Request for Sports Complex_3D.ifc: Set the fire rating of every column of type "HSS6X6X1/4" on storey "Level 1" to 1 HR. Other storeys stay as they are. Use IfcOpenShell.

First a look at what the model holds.

```python
import ifcopenshell
import ifcopenshell.util.element

model = ifcopenshell.open("Sports Complex_3D.ifc")
print(model.schema)
storey = next(s for s in model.by_type("IfcBuildingStorey") if s.Name == "Level 1")
columns = [e for e in ifcopenshell.util.element.get_decomposition(storey) if e.is_a("IfcColumn")]
seen = {}
for e in columns:
    element_type = ifcopenshell.util.element.get_type(e)
    key = (element_type.Name if element_type != e and element_type else None, ifcopenshell.util.element.get_pset(e, "Pset_ColumnCommon", "FireRating"))
    seen[key] = seen.get(key, 0) + 1
for (name, value), count in sorted(seen.items(), key=str):
    print(count, "x", name, "|", value)
```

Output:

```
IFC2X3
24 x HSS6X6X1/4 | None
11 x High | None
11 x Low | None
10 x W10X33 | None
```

```python
import ifcopenshell
import ifcopenshell.api.pset
import ifcopenshell.util.element

model = ifcopenshell.open("Sports Complex_3D.ifc")

storey = next(s for s in model.by_type("IfcBuildingStorey") if s.Name == "Level 1")
columns = [e for e in ifcopenshell.util.element.get_decomposition(storey) if e.is_a("IfcColumn")]

count = 0
for e in columns:
    element_type = ifcopenshell.util.element.get_type(e)
    if element_type in (None, e) or element_type.Name != "HSS6X6X1/4":
        continue
    # add_pset returns the element's existing set when there is one.
    pset = ifcopenshell.api.pset.add_pset(model, product=e, name="Pset_ColumnCommon")
    ifcopenshell.api.pset.edit_pset(model, pset=pset, properties={"FireRating": "1 HR"})
    count += 1

print(count, "columns updated")

model.write("Sports Complex_3D_edited.ifc")
```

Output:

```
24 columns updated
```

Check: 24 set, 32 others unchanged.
